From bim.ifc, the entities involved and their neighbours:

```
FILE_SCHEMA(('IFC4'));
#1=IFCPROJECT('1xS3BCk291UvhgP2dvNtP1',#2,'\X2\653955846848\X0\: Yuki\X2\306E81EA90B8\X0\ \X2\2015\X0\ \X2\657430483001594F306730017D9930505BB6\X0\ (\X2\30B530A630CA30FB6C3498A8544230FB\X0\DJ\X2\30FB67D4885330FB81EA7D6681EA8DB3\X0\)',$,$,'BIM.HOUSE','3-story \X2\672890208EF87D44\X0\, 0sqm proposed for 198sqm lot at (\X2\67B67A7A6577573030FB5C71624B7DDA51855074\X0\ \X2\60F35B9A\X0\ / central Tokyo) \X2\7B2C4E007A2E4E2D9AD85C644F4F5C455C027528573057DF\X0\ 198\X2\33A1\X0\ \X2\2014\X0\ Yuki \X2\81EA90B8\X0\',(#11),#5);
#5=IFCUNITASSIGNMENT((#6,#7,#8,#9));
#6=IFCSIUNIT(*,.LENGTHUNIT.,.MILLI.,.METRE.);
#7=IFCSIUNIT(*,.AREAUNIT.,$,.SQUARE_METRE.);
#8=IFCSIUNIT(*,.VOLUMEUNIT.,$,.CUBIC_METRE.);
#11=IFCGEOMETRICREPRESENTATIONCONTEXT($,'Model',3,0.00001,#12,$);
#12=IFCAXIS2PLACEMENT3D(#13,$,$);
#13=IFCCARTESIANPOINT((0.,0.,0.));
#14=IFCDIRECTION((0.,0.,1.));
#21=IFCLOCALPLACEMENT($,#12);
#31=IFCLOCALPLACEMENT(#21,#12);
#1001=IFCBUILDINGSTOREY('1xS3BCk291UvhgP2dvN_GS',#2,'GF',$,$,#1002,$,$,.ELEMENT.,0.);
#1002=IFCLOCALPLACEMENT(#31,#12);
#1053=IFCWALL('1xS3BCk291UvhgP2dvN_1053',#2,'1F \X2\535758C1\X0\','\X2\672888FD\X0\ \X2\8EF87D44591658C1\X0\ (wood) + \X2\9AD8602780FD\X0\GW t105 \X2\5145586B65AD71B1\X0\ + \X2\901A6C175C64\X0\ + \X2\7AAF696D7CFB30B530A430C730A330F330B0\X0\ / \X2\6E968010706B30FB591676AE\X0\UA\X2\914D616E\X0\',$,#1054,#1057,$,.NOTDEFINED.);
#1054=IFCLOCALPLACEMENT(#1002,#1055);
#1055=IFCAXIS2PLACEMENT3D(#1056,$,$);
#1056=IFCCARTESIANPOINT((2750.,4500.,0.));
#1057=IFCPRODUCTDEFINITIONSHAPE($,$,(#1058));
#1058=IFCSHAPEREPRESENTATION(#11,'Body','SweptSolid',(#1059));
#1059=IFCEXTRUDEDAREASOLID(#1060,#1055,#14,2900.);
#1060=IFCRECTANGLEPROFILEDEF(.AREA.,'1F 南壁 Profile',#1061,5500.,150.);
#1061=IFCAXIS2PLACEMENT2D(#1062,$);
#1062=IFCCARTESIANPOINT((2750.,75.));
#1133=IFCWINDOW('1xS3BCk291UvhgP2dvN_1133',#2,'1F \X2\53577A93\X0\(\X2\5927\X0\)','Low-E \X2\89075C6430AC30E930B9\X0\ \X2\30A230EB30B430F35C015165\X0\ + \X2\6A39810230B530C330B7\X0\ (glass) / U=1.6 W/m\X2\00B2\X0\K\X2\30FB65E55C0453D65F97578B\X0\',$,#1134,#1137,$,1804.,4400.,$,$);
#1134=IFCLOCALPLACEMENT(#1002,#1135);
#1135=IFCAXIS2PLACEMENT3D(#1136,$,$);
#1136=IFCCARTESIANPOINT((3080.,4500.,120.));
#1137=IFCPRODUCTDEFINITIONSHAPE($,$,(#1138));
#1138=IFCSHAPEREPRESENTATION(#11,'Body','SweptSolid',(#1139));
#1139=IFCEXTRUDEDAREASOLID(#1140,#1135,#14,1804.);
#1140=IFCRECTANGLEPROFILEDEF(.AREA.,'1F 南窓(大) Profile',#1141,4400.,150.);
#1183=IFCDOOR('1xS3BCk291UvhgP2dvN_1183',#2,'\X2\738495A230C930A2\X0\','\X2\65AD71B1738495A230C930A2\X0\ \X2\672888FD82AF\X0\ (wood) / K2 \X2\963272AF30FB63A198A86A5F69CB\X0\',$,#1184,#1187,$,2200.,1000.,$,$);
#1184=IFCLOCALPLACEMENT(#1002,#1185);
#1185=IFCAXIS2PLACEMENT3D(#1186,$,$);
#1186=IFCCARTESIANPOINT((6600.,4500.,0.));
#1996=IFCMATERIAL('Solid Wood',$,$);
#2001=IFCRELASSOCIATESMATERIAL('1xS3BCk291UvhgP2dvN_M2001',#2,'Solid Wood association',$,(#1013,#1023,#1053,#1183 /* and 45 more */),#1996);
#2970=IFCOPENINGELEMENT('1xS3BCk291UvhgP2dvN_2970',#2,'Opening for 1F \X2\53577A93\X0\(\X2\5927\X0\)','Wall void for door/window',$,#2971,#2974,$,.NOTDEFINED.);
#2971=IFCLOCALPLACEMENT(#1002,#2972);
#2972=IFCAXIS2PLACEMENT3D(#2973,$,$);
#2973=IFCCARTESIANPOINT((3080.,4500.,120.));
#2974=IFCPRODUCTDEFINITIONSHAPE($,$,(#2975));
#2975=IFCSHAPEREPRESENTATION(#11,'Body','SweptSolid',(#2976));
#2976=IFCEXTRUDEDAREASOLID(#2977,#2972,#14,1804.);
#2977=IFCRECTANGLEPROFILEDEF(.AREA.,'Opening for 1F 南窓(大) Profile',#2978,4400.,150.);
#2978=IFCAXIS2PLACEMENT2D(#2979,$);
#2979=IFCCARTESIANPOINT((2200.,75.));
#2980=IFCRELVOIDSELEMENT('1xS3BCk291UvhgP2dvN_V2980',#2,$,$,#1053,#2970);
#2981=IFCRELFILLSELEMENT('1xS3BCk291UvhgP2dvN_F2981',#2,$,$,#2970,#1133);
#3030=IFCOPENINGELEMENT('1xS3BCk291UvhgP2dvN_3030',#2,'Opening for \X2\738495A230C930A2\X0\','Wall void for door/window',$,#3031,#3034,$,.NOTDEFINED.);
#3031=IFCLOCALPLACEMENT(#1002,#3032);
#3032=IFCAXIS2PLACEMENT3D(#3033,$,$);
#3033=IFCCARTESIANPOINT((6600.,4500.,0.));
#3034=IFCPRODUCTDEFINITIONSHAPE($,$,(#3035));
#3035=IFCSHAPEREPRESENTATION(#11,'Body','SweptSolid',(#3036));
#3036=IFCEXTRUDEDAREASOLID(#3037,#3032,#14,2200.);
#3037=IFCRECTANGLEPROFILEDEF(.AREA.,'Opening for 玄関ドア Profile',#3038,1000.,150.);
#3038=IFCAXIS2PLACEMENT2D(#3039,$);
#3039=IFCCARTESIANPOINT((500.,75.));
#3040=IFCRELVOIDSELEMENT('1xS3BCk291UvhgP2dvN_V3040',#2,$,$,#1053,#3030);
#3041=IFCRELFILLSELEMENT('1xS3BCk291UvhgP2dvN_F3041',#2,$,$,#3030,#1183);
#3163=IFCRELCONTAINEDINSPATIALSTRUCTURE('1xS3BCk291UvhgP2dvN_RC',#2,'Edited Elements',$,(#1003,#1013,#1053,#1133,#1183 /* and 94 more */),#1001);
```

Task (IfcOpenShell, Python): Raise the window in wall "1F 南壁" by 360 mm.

```python
import numpy as np
import ifcopenshell
import ifcopenshell.api.geometry
import ifcopenshell.util.placement
import ifcopenshell.util.unit

model = ifcopenshell.open("bim.ifc")
unit_scale = ifcopenshell.util.unit.calculate_unit_scale(model)

window = model.by_id(1133)
opening = window.FillsVoids[0].RelatingOpeningElement
dz = 360.0

shift = np.array([0.0, 0.0, dz])
# The window is not placed relative to its opening, so move both.
for product in (opening, window):
    matrix = ifcopenshell.util.placement.get_local_placement(product.ObjectPlacement)
    matrix[:3, 3] += shift
    ifcopenshell.api.geometry.edit_object_placement(model, product=product, matrix=matrix, is_si=False)

print(f"moved by {dz * unit_scale:+.3f} m")

model.write("bim-out.ifc")
```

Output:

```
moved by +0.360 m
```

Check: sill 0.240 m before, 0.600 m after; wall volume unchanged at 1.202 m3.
